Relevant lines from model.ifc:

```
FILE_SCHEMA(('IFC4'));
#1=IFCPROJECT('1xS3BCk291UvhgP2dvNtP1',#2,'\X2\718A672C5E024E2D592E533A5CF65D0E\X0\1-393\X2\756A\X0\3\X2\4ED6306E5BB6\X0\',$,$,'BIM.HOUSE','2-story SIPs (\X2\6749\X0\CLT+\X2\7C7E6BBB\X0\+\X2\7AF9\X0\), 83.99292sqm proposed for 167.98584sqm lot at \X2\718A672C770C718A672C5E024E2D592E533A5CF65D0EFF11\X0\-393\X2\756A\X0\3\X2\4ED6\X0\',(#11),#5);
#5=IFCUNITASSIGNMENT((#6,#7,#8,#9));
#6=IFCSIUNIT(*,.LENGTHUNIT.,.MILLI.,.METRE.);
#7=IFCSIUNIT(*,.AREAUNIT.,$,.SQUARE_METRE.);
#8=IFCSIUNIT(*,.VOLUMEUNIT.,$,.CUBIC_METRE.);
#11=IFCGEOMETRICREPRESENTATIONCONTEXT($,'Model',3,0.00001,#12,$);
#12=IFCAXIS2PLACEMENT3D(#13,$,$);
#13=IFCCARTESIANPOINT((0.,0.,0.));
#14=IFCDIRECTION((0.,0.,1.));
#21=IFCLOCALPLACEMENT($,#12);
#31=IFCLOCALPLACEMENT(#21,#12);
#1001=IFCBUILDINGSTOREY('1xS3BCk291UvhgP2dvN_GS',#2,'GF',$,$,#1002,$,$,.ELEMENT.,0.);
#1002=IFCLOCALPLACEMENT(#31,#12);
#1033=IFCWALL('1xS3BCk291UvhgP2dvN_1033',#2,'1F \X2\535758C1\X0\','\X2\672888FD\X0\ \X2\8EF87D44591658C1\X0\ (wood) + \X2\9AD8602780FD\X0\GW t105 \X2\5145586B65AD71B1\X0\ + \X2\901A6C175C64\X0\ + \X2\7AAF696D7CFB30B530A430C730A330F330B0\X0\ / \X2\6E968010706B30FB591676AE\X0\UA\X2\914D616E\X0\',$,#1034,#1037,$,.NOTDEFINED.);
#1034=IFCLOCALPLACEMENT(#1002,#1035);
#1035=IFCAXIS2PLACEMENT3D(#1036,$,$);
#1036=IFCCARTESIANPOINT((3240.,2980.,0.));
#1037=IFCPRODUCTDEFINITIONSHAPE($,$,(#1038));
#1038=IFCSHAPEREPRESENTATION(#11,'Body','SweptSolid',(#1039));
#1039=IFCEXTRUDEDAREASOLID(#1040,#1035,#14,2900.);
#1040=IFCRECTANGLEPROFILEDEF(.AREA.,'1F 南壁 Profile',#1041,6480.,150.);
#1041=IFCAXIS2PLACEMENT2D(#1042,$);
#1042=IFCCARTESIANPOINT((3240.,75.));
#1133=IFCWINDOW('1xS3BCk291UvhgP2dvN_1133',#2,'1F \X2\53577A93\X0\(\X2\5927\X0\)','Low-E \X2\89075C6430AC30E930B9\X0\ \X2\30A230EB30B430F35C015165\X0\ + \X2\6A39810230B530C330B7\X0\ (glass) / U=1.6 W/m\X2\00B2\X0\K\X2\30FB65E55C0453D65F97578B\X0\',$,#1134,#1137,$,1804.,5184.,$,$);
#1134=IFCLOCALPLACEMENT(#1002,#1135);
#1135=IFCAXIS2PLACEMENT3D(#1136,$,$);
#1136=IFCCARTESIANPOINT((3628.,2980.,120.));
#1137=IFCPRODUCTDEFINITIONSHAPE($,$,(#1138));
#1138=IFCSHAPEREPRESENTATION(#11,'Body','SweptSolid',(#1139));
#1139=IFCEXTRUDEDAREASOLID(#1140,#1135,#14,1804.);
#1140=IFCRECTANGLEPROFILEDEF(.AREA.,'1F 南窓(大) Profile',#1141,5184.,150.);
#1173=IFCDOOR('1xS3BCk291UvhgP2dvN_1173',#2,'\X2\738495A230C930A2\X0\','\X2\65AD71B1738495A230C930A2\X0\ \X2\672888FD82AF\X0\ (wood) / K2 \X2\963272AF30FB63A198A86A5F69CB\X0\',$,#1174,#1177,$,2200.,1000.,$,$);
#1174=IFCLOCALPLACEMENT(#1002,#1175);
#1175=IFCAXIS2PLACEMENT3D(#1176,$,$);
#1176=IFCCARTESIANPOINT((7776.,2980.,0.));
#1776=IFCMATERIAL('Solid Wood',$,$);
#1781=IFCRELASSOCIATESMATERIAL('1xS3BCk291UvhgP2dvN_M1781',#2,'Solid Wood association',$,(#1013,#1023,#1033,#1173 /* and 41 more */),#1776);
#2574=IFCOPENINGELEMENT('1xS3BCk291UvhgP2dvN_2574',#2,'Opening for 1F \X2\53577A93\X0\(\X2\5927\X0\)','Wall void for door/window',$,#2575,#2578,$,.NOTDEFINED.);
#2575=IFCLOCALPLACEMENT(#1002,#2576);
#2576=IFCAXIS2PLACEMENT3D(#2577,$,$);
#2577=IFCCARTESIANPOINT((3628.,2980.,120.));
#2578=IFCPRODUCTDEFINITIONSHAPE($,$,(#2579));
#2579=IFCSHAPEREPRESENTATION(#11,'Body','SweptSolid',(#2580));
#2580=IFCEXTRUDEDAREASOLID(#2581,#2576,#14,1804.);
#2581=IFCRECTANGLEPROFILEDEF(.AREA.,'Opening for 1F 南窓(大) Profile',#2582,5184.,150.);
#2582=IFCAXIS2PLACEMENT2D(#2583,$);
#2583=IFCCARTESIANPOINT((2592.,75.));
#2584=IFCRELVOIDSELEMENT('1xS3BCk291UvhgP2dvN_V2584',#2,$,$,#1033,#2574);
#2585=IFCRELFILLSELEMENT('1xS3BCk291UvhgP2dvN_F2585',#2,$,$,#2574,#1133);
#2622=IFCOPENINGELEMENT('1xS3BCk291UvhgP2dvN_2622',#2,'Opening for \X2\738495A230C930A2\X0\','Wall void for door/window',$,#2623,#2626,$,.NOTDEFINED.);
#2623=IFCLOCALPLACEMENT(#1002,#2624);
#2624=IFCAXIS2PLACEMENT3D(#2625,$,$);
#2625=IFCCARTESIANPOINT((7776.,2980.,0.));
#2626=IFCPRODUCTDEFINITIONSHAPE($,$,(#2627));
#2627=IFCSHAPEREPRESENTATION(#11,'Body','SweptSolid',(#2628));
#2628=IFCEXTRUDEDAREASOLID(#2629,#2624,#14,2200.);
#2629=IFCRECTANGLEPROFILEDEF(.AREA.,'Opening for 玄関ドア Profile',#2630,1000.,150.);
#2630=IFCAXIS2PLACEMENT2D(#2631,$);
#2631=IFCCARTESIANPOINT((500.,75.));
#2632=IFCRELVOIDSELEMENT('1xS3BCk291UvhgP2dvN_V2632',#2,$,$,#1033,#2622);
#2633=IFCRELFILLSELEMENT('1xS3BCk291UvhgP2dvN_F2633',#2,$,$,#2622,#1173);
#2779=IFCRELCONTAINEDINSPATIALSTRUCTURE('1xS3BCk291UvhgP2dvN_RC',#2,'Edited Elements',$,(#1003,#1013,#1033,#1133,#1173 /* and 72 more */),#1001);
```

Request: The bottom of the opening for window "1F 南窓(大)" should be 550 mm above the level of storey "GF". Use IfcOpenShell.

```python
import numpy as np
import ifcopenshell
import ifcopenshell.api.geometry
import ifcopenshell.geom
import ifcopenshell.util.element
import ifcopenshell.util.placement
import ifcopenshell.util.shape
import ifcopenshell.util.unit

model = ifcopenshell.open("model.ifc")
unit_scale = ifcopenshell.util.unit.calculate_unit_scale(model)

window = model.by_guid("1xS3BCk291UvhgP2dvN_1133")
opening = window.FillsVoids[0].RelatingOpeningElement
storey = ifcopenshell.util.element.get_container(window, ifc_class="IfcBuildingStorey")
level = ifcopenshell.util.placement.get_local_placement(storey.ObjectPlacement)[2, 3]

# The opening's origin need not be at the sill, so measure its lowest point.
shape = ifcopenshell.geom.create_shape(ifcopenshell.geom.settings(), opening)
bottom = ifcopenshell.util.shape.get_shape_bottom_elevation(shape, shape.geometry) / unit_scale
dz = level + 0.55 / unit_scale - bottom

shift = np.array([0.0, 0.0, dz])
# The window is not placed relative to its opening, so move both.
for product in (opening, window):
    matrix = ifcopenshell.util.placement.get_local_placement(product.ObjectPlacement)
    matrix[:3, 3] += shift
    ifcopenshell.api.geometry.edit_object_placement(model, product=product, matrix=matrix, is_si=False)

print(f"moved by {dz * unit_scale:+.3f} m")

model.write("model_updated.ifc")
```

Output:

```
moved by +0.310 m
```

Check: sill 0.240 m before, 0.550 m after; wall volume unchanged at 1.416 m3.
